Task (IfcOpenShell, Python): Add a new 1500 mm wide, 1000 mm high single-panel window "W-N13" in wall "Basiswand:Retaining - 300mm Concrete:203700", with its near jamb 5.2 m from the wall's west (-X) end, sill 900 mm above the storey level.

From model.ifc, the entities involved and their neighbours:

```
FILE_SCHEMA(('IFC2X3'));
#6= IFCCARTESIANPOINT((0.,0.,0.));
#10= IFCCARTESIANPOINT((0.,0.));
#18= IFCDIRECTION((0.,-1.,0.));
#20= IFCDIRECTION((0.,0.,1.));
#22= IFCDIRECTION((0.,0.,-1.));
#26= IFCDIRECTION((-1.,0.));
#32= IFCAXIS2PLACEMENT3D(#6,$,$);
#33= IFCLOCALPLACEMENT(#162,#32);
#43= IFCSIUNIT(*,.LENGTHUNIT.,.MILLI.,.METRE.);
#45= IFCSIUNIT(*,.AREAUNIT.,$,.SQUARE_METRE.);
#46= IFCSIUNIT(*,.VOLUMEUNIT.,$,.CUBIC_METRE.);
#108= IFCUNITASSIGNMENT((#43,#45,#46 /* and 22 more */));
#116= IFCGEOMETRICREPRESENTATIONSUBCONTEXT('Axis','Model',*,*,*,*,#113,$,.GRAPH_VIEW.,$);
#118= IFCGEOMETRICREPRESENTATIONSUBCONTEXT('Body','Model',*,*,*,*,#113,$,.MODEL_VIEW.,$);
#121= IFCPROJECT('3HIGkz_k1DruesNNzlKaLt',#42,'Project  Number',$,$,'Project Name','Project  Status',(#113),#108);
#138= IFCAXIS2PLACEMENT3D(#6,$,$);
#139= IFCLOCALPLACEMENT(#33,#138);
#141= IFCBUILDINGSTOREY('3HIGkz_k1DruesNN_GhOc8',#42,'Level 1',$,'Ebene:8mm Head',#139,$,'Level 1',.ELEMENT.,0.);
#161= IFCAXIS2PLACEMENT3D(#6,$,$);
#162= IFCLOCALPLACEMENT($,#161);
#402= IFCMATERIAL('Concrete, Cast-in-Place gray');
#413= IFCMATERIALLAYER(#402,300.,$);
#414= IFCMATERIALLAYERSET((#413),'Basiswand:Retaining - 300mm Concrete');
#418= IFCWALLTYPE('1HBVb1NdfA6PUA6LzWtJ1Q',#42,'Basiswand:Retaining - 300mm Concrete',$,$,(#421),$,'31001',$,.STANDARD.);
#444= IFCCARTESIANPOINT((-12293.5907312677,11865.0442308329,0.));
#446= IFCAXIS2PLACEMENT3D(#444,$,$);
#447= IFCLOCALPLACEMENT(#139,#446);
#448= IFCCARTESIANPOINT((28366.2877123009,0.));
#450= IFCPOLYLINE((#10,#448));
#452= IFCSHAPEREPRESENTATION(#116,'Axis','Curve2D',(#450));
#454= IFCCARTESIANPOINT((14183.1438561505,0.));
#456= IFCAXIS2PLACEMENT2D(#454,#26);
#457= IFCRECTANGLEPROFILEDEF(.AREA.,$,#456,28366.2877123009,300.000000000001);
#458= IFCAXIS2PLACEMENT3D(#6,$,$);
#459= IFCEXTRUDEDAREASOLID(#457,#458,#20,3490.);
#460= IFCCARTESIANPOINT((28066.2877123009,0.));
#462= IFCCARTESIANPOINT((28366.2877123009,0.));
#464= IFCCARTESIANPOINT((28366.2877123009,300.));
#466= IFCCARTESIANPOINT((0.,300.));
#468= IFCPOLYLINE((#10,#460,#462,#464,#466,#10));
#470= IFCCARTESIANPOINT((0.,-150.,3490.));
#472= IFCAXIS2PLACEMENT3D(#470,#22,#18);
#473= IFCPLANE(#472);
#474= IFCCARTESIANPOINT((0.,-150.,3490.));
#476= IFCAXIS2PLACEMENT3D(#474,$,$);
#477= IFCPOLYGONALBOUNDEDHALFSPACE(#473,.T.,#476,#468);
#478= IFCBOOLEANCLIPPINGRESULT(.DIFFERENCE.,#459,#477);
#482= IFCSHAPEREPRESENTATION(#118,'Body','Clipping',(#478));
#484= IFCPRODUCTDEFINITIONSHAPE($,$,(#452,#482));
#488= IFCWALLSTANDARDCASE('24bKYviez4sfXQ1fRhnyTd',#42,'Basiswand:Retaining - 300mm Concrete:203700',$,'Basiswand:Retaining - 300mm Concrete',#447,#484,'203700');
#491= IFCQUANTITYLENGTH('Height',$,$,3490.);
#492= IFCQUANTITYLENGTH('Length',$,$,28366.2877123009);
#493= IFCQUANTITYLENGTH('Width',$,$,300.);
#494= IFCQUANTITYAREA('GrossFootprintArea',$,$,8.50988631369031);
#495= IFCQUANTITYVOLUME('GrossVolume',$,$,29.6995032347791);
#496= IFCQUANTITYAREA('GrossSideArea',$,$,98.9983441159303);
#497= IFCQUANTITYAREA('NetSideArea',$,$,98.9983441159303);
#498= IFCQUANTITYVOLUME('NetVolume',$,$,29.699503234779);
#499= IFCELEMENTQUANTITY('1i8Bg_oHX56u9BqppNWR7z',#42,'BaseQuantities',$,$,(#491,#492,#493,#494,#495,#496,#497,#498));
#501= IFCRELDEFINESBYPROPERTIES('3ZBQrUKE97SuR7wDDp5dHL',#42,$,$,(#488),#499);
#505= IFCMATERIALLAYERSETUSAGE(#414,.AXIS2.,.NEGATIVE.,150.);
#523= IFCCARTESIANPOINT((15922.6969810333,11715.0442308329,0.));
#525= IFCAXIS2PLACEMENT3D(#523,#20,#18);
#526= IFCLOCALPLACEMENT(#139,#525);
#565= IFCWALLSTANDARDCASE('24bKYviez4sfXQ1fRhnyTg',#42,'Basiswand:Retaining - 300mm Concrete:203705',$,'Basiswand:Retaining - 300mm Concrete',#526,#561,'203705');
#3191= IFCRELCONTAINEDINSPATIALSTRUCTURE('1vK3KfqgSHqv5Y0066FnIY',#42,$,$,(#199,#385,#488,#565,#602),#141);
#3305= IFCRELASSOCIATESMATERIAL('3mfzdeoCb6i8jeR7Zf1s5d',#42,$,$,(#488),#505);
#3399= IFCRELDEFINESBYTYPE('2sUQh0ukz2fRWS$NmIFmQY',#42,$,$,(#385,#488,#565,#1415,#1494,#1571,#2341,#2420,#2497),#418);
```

```python
import numpy as np
import ifcopenshell
import ifcopenshell.api.feature
import ifcopenshell.api.geometry
import ifcopenshell.api.pset
import ifcopenshell.api.root
import ifcopenshell.api.spatial
import ifcopenshell.api.type
import ifcopenshell.geom
import ifcopenshell.util.element
import ifcopenshell.util.placement
import ifcopenshell.util.representation
import ifcopenshell.util.shape
import ifcopenshell.util.unit

model = ifcopenshell.open("model.ifc")
unit_scale = ifcopenshell.util.unit.calculate_unit_scale(model)
area_scale = ifcopenshell.util.unit.calculate_unit_scale(model, "AREAUNIT")
volume_scale = ifcopenshell.util.unit.calculate_unit_scale(model, "VOLUMEUNIT")
settings = ifcopenshell.geom.settings()


def volume(element):
    """Net volume in cubic metres, openings subtracted."""
    shape = ifcopenshell.geom.create_shape(settings, element)
    return ifcopenshell.util.shape.get_volume(shape.geometry)


wall = model.by_guid("24bKYviez4sfXQ1fRhnyTd")
storey = ifcopenshell.util.element.get_container(wall, ifc_class="IfcBuildingStorey")
context = ifcopenshell.util.representation.get_context(model, "Model", "Body", "MODEL_VIEW")
before = volume(wall)

width, height, from_end, sill = 1.5, 1, 5.2, 0.9  # metres

# The wall runs along its own X axis, and the end named is its -X end.
wall_shape = ifcopenshell.geom.create_shape(settings, wall)
x, y, z = ifcopenshell.util.shape.get_vertices(wall_shape.geometry).T
start = x.min() + from_end
face, thickness = float(y.min()), float(y.max() - y.min())
wall_matrix = ifcopenshell.util.placement.get_local_placement(wall.ObjectPlacement)
level = ifcopenshell.util.placement.get_local_placement(storey.ObjectPlacement)[2, 3]


def in_wall(x, y):
    """Placement at x, y metres in the wall's axes, at sill height."""
    matrix = wall_matrix.copy()
    matrix[:, 3] = wall_matrix @ np.array([x / unit_scale, y / unit_scale, 0.0, 1.0])
    matrix[2, 3] = level + sill / unit_scale
    return matrix


# Opening: a box that overshoots both wall faces by 50 mm.
opening = ifcopenshell.api.root.create_entity(model, ifc_class="IfcOpeningElement")
box = ifcopenshell.api.geometry.add_wall_representation(
    model, context=context, length=width, height=height, thickness=thickness + 0.1
)
ifcopenshell.api.geometry.assign_representation(model, product=opening, representation=box)
ifcopenshell.api.geometry.edit_object_placement(model, product=opening, matrix=in_wall(start, face - 0.05), is_si=False)
ifcopenshell.api.feature.add_feature(model, feature=opening, element=wall)

window = ifcopenshell.api.root.create_entity(model, ifc_class="IfcWindow", name="W-N13")
window.OverallWidth, window.OverallHeight = width / unit_scale, height / unit_scale
body = ifcopenshell.api.geometry.add_window_representation(
    model,
    context=context,
    overall_width=window.OverallWidth,
    overall_height=window.OverallHeight,
    partition_type="SINGLE_PANEL",
)
ifcopenshell.api.geometry.assign_representation(model, product=window, representation=body)
ifcopenshell.api.spatial.assign_container(model, products=[window], relating_structure=storey)
fills = ifcopenshell.api.feature.add_filling(model, opening=opening, element=window)
fills.OwnerHistory = window.OwnerHistory  # required in IFC2X3

# IFC2X3 keeps the operation on the window style.
style = ifcopenshell.api.root.create_entity(model, ifc_class="IfcWindowStyle", name="W-N13")
style.OperationType, style.ConstructionType = "SINGLE_PANEL", "NOTDEFINED"
style.ParameterTakesPrecedence = style.Sizeable = False
ifcopenshell.api.type.assign_type(model, related_objects=[window], relating_type=style)

# Centre the window in the wall's thickness.
ifcopenshell.api.geometry.edit_object_placement(model, product=window, matrix=in_wall(start, face), is_si=False)
window_shape = ifcopenshell.geom.create_shape(settings, window)
depth = ifcopenshell.util.shape.get_vertices(window_shape.geometry)[:, 1]
offset = face + thickness / 2 - (depth.min() + depth.max()) / 2
ifcopenshell.api.geometry.edit_object_placement(model, product=window, matrix=in_wall(start, offset), is_si=False)

after = volume(wall)

# Update the wall's stored quantities.
qto = model.by_id(ifcopenshell.util.element.get_pset(wall, "BaseQuantities", should_inherit=False)["id"])
ifcopenshell.api.pset.edit_qto(model, qto=qto, properties={
    "NetSideArea": after / thickness / area_scale,
    "NetVolume": after / volume_scale,
})

print(f"wall volume {before:.3f} -> {after:.3f} m3")

model.write("model_rev.ifc")
```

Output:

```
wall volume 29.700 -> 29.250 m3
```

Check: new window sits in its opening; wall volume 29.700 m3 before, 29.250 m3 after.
